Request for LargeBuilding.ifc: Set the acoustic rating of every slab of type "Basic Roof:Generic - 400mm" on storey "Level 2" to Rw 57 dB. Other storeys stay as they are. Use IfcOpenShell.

First a look at what the model holds.

```python
import ifcopenshell
import ifcopenshell.util.element

model = ifcopenshell.open("LargeBuilding.ifc")
print(model.schema)
storey = next(s for s in model.by_type("IfcBuildingStorey") if s.Name == "Level 2")
slabs = [e for e in ifcopenshell.util.element.get_decomposition(storey) if e.is_a("IfcSlab")]
seen = {}
for e in slabs:
    element_type = ifcopenshell.util.element.get_type(e)
    key = (element_type.Name if element_type != e and element_type else None, ifcopenshell.util.element.get_pset(e, "Pset_SlabCommon", "AcousticRating"))
    seen[key] = seen.get(key, 0) + 1
for (name, value), count in sorted(seen.items(), key=str):
    print(count, "x", name, "|", value)
```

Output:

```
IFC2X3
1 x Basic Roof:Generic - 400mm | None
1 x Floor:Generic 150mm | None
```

```python
import ifcopenshell
import ifcopenshell.api.pset
import ifcopenshell.util.element

model = ifcopenshell.open("LargeBuilding.ifc")

storey = next(s for s in model.by_type("IfcBuildingStorey") if s.Name == "Level 2")
slabs = [e for e in ifcopenshell.util.element.get_decomposition(storey) if e.is_a("IfcSlab")]

count = 0
for e in slabs:
    element_type = ifcopenshell.util.element.get_type(e)
    if element_type in (None, e) or element_type.Name != "Basic Roof:Generic - 400mm":
        continue
    # add_pset returns the element's existing set when there is one.
    pset = ifcopenshell.api.pset.add_pset(model, product=e, name="Pset_SlabCommon")
    ifcopenshell.api.pset.edit_pset(model, pset=pset, properties={"AcousticRating": "Rw 57 dB"})
    count += 1

print(count, "slabs updated")

model.write("LargeBuilding_v2.ifc")
```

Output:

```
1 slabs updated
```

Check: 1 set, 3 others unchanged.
